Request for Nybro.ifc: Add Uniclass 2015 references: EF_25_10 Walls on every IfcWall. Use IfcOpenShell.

First a look at what the model holds.

```python
import ifcopenshell

model = ifcopenshell.open("Nybro.ifc")
print(model.schema)
print("classifications:", [c.Name for c in model.by_type("IfcClassification")])
for ifc_class in ("IfcDoor", "IfcRoof", "IfcStair", "IfcWall", "IfcWindow"):
    print(ifc_class, len(model.by_type(ifc_class)))
```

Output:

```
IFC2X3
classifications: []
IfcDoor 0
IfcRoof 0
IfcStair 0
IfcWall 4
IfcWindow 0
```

```python
import ifcopenshell
import ifcopenshell.api.classification

model = ifcopenshell.open("Nybro.ifc")

# IFC2X3 requires Source and Edition and has no link from the project to the system.
system = model.create_entity("IfcClassification", Source="NBS", Edition="2015", Name="Uniclass 2015")

codes = {
    "IfcWall": ("EF_25_10", "Walls"),
}
for ifc_class, (code, name) in codes.items():
    products = model.by_type(ifc_class)
    ifcopenshell.api.classification.add_reference(
        model, products=products, classification=system, identification=code, name=name
    )
    print(code, len(products))

model.write("Nybro_edited.ifc")
```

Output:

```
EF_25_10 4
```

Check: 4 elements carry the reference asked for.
